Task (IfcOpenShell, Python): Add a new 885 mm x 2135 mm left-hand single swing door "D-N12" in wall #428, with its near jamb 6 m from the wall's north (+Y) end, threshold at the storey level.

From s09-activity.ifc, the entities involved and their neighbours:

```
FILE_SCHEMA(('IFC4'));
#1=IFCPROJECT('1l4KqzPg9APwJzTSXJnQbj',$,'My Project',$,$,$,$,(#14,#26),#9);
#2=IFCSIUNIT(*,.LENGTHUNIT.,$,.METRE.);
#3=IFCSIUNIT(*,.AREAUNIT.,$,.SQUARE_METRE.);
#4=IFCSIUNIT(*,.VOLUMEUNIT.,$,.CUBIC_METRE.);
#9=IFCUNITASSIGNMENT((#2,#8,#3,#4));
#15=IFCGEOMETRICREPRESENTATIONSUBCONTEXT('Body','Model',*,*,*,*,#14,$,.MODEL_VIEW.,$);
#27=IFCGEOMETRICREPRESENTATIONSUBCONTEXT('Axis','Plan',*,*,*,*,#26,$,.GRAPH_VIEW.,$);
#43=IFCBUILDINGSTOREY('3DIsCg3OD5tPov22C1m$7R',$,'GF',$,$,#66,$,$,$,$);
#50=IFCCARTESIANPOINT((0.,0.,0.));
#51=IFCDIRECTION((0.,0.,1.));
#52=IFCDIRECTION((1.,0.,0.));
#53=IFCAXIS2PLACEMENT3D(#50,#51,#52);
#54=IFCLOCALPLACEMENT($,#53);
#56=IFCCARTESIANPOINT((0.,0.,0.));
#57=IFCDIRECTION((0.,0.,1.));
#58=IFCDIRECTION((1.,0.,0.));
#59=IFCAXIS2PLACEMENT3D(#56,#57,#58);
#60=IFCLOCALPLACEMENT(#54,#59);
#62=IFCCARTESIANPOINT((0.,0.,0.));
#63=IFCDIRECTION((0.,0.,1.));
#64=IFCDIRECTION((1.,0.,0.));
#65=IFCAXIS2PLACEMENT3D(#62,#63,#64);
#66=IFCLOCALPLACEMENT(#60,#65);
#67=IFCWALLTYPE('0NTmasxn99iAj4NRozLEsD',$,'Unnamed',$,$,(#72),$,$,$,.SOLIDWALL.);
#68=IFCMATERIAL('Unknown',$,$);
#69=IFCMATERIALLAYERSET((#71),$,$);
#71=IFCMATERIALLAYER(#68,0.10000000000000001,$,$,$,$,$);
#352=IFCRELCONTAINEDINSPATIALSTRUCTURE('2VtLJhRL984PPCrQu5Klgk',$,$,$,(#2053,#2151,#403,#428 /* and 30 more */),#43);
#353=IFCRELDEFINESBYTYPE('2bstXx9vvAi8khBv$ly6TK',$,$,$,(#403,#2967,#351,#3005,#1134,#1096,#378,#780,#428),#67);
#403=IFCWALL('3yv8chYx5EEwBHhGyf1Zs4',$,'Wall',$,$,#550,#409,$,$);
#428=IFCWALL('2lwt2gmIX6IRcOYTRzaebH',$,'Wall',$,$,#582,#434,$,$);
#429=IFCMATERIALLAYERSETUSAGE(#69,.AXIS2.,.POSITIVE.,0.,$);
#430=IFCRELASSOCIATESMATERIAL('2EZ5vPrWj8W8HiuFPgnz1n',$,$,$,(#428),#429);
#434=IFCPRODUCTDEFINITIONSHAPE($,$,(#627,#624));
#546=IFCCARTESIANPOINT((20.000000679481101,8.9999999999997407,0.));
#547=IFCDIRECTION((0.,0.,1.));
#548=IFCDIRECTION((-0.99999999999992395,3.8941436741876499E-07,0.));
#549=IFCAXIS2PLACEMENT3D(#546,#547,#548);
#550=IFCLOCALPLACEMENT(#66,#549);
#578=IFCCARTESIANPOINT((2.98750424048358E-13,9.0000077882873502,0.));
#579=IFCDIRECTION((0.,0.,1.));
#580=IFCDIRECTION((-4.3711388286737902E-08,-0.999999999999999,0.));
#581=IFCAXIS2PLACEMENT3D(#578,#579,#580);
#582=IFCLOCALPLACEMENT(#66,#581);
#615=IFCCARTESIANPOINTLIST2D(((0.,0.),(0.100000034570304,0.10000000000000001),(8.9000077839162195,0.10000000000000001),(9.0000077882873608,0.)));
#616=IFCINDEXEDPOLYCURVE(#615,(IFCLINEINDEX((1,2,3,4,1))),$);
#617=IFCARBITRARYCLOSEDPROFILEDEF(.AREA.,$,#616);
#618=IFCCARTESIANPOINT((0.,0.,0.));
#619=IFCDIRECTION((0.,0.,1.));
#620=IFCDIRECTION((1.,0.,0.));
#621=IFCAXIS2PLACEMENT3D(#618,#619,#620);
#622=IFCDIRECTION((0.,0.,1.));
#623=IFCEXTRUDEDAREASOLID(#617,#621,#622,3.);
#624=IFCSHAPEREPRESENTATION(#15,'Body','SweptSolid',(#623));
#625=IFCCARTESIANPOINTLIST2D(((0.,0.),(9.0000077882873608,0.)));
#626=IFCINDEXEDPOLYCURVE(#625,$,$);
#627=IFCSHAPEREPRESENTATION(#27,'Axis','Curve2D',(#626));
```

```python
import numpy as np
import ifcopenshell
import ifcopenshell.api.feature
import ifcopenshell.api.geometry
import ifcopenshell.api.root
import ifcopenshell.api.spatial
import ifcopenshell.geom
import ifcopenshell.util.element
import ifcopenshell.util.placement
import ifcopenshell.util.representation
import ifcopenshell.util.shape
import ifcopenshell.util.unit

model = ifcopenshell.open("s09-activity.ifc")
unit_scale = ifcopenshell.util.unit.calculate_unit_scale(model)
settings = ifcopenshell.geom.settings()


def volume(element):
    """Net volume in cubic metres, openings subtracted."""
    shape = ifcopenshell.geom.create_shape(settings, element)
    return ifcopenshell.util.shape.get_volume(shape.geometry)


wall = model.by_id(428)
storey = ifcopenshell.util.element.get_container(wall, ifc_class="IfcBuildingStorey")
context = ifcopenshell.util.representation.get_context(model, "Model", "Body", "MODEL_VIEW")
before = volume(wall)

width, height, from_end, sill = 0.885, 2.135, 6, 0.0  # metres

# The wall runs along its own X axis, and the end named is its -X end.
wall_shape = ifcopenshell.geom.create_shape(settings, wall)
x, y, z = ifcopenshell.util.shape.get_vertices(wall_shape.geometry).T
start = x.min() + from_end
face, thickness = float(y.min()), float(y.max() - y.min())
wall_matrix = ifcopenshell.util.placement.get_local_placement(wall.ObjectPlacement)
level = ifcopenshell.util.placement.get_local_placement(storey.ObjectPlacement)[2, 3]


def in_wall(x, y):
    """Placement at x, y metres in the wall's axes, at sill height."""
    matrix = wall_matrix.copy()
    matrix[:, 3] = wall_matrix @ np.array([x / unit_scale, y / unit_scale, 0.0, 1.0])
    matrix[2, 3] = level + sill / unit_scale
    return matrix


# Opening: a box that overshoots both wall faces by 50 mm.
opening = ifcopenshell.api.root.create_entity(model, ifc_class="IfcOpeningElement", predefined_type="OPENING")
box = ifcopenshell.api.geometry.add_wall_representation(
    model, context=context, length=width, height=height, thickness=thickness + 0.1
)
ifcopenshell.api.geometry.assign_representation(model, product=opening, representation=box)
ifcopenshell.api.geometry.edit_object_placement(model, product=opening, matrix=in_wall(start, face - 0.05), is_si=False)
ifcopenshell.api.feature.add_feature(model, feature=opening, element=wall)

door = ifcopenshell.api.root.create_entity(model, ifc_class="IfcDoor", name="D-N12", predefined_type="DOOR")
door.OverallWidth, door.OverallHeight = width / unit_scale, height / unit_scale
door.OperationType = "SINGLE_SWING_LEFT"
body = ifcopenshell.api.geometry.add_door_representation(
    model,
    context=context,
    overall_width=door.OverallWidth,
    overall_height=door.OverallHeight,
    operation_type="SINGLE_SWING_LEFT",
    lining_properties={"LiningDepth": thickness / unit_scale, "ThresholdDepth": thickness / unit_scale},
)
ifcopenshell.api.geometry.assign_representation(model, product=door, representation=body)
ifcopenshell.api.spatial.assign_container(model, products=[door], relating_structure=storey)
ifcopenshell.api.feature.add_filling(model, opening=opening, element=door)

# The lining spans the wall, so the door starts at the wall face.
ifcopenshell.api.geometry.edit_object_placement(model, product=door, matrix=in_wall(start, face), is_si=False)

after = volume(wall)

print(f"wall volume {before:.3f} -> {after:.3f} m3")

model.write("s09-activity_updated.ifc")
```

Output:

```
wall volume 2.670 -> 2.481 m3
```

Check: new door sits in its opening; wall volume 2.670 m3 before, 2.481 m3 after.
